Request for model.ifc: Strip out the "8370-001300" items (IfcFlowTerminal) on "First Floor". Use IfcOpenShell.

First a look at what the model holds.

```python
import ifcopenshell
import ifcopenshell.util.element

model = ifcopenshell.open("model.ifc")
print(model.schema)
storey = next(s for s in model.by_type("IfcBuildingStorey") if s.Name == "First Floor")
terminals = [e for e in ifcopenshell.util.element.get_decomposition(storey) if e.is_a("IfcFlowTerminal")]
seen = {}
for e in terminals:
    element_type = ifcopenshell.util.element.get_type(e)
    name = element_type.Name if element_type not in (None, e) else None
    seen[name] = seen.get(name, 0) + 1
for name, count in sorted(seen.items(), key=str):
    print(count, "x", name)
```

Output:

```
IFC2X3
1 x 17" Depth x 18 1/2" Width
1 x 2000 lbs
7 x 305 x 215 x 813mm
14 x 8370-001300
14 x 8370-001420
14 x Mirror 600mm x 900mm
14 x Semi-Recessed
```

```python
import ifcopenshell
import ifcopenshell.api.root
import ifcopenshell.util.element

model = ifcopenshell.open("model.ifc")

storey = next(s for s in model.by_type("IfcBuildingStorey") if s.Name == "First Floor")
terminals = [e for e in ifcopenshell.util.element.get_decomposition(storey) if e.is_a("IfcFlowTerminal")]
targets = [e for e in terminals if (t := ifcopenshell.util.element.get_type(e)) not in (None, e) and t.Name == "8370-001300"]

for e in targets:
    ifcopenshell.api.root.remove_product(model, product=e)
print(len(targets), "removed")

model.write("model_v2.ifc")
```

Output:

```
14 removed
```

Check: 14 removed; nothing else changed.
